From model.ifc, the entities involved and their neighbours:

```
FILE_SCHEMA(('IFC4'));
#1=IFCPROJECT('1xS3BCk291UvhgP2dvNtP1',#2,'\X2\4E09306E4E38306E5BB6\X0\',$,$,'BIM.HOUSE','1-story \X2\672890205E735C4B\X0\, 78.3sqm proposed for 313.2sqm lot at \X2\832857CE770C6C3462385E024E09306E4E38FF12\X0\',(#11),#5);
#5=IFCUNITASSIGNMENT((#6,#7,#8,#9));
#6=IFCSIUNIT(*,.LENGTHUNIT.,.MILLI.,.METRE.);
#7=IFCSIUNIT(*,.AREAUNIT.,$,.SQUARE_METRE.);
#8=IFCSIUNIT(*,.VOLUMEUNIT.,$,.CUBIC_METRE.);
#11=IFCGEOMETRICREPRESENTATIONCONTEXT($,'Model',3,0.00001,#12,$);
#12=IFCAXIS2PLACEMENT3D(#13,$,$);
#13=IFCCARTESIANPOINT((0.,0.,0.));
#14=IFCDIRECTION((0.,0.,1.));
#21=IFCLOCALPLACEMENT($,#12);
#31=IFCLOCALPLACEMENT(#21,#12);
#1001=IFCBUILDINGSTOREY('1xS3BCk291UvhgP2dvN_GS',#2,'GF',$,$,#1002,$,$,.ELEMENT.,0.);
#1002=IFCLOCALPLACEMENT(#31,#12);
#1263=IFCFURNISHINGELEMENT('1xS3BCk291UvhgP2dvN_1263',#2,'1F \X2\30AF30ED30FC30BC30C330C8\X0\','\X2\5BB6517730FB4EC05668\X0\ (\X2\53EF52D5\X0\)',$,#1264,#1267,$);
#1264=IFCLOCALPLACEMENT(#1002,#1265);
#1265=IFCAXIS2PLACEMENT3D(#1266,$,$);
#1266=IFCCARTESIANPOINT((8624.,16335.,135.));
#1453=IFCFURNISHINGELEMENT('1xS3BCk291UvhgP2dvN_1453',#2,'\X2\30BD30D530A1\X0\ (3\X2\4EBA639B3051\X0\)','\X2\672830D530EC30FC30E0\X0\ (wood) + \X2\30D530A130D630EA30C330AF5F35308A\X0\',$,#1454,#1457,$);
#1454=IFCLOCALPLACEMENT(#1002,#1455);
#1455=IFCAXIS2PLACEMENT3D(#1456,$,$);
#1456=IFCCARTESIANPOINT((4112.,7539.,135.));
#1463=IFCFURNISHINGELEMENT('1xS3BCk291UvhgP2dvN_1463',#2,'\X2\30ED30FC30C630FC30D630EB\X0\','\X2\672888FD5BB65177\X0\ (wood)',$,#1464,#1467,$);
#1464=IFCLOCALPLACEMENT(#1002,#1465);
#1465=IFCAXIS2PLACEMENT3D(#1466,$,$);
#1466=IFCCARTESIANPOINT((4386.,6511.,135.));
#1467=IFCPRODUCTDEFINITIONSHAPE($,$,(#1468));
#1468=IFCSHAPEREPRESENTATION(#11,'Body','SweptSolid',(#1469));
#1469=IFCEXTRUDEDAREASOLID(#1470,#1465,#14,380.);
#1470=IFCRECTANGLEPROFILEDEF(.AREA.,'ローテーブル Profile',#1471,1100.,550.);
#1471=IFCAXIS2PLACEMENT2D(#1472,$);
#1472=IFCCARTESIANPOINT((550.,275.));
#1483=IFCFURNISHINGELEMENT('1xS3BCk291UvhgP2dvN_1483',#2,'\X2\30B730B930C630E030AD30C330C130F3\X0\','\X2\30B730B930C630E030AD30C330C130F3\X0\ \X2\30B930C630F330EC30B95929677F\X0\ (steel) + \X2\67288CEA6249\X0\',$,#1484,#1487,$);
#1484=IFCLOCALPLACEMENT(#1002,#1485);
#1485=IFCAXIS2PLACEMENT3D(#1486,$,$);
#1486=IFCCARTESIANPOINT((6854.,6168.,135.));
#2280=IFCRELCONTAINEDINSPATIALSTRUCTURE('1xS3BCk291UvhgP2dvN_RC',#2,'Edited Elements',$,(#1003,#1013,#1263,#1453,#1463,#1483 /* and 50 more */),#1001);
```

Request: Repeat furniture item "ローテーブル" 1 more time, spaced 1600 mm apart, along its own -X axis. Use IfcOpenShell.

```python
import ifcopenshell
import ifcopenshell.api.geometry
import ifcopenshell.api.root
import ifcopenshell.util.element
import ifcopenshell.util.placement
import ifcopenshell.util.unit

model = ifcopenshell.open("model.ifc")
unit_scale = ifcopenshell.util.unit.calculate_unit_scale(model)


def reuse_history(source, copy):
    """copy_class also copies each property set's owner history, people and application; keep the originals."""
    for rel in copy.IsDefinedBy:
        if rel.is_a("IfcRelDefinesByProperties") and (history := rel.RelatingPropertyDefinition.OwnerHistory):
            rel.RelatingPropertyDefinition.OwnerHistory = source.OwnerHistory
            ifcopenshell.util.element.remove_deep2(model, history)


source = model.by_guid("1xS3BCk291UvhgP2dvN_1463")
base = ifcopenshell.util.placement.get_local_placement(source.ObjectPlacement)
step = -base[:3, 0] * 1.6 / unit_scale

for i in range(1, 2):
    copy = ifcopenshell.api.root.copy_class(model, product=source)
    copy.Representation = ifcopenshell.util.element.copy_deep(
        model, source.Representation, exclude=["IfcGeometricRepresentationContext", "IfcRepresentationMap"]
    )
    reuse_history(source, copy)
    matrix = base.copy()
    matrix[:3, 3] += i * step
    print("added at", matrix[:3, 3].round(3) + 0.0)
    ifcopenshell.api.geometry.edit_object_placement(model, product=copy, matrix=matrix, is_si=False)

model.write("model_rev.ifc")
```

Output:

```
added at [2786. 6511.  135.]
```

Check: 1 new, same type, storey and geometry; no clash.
